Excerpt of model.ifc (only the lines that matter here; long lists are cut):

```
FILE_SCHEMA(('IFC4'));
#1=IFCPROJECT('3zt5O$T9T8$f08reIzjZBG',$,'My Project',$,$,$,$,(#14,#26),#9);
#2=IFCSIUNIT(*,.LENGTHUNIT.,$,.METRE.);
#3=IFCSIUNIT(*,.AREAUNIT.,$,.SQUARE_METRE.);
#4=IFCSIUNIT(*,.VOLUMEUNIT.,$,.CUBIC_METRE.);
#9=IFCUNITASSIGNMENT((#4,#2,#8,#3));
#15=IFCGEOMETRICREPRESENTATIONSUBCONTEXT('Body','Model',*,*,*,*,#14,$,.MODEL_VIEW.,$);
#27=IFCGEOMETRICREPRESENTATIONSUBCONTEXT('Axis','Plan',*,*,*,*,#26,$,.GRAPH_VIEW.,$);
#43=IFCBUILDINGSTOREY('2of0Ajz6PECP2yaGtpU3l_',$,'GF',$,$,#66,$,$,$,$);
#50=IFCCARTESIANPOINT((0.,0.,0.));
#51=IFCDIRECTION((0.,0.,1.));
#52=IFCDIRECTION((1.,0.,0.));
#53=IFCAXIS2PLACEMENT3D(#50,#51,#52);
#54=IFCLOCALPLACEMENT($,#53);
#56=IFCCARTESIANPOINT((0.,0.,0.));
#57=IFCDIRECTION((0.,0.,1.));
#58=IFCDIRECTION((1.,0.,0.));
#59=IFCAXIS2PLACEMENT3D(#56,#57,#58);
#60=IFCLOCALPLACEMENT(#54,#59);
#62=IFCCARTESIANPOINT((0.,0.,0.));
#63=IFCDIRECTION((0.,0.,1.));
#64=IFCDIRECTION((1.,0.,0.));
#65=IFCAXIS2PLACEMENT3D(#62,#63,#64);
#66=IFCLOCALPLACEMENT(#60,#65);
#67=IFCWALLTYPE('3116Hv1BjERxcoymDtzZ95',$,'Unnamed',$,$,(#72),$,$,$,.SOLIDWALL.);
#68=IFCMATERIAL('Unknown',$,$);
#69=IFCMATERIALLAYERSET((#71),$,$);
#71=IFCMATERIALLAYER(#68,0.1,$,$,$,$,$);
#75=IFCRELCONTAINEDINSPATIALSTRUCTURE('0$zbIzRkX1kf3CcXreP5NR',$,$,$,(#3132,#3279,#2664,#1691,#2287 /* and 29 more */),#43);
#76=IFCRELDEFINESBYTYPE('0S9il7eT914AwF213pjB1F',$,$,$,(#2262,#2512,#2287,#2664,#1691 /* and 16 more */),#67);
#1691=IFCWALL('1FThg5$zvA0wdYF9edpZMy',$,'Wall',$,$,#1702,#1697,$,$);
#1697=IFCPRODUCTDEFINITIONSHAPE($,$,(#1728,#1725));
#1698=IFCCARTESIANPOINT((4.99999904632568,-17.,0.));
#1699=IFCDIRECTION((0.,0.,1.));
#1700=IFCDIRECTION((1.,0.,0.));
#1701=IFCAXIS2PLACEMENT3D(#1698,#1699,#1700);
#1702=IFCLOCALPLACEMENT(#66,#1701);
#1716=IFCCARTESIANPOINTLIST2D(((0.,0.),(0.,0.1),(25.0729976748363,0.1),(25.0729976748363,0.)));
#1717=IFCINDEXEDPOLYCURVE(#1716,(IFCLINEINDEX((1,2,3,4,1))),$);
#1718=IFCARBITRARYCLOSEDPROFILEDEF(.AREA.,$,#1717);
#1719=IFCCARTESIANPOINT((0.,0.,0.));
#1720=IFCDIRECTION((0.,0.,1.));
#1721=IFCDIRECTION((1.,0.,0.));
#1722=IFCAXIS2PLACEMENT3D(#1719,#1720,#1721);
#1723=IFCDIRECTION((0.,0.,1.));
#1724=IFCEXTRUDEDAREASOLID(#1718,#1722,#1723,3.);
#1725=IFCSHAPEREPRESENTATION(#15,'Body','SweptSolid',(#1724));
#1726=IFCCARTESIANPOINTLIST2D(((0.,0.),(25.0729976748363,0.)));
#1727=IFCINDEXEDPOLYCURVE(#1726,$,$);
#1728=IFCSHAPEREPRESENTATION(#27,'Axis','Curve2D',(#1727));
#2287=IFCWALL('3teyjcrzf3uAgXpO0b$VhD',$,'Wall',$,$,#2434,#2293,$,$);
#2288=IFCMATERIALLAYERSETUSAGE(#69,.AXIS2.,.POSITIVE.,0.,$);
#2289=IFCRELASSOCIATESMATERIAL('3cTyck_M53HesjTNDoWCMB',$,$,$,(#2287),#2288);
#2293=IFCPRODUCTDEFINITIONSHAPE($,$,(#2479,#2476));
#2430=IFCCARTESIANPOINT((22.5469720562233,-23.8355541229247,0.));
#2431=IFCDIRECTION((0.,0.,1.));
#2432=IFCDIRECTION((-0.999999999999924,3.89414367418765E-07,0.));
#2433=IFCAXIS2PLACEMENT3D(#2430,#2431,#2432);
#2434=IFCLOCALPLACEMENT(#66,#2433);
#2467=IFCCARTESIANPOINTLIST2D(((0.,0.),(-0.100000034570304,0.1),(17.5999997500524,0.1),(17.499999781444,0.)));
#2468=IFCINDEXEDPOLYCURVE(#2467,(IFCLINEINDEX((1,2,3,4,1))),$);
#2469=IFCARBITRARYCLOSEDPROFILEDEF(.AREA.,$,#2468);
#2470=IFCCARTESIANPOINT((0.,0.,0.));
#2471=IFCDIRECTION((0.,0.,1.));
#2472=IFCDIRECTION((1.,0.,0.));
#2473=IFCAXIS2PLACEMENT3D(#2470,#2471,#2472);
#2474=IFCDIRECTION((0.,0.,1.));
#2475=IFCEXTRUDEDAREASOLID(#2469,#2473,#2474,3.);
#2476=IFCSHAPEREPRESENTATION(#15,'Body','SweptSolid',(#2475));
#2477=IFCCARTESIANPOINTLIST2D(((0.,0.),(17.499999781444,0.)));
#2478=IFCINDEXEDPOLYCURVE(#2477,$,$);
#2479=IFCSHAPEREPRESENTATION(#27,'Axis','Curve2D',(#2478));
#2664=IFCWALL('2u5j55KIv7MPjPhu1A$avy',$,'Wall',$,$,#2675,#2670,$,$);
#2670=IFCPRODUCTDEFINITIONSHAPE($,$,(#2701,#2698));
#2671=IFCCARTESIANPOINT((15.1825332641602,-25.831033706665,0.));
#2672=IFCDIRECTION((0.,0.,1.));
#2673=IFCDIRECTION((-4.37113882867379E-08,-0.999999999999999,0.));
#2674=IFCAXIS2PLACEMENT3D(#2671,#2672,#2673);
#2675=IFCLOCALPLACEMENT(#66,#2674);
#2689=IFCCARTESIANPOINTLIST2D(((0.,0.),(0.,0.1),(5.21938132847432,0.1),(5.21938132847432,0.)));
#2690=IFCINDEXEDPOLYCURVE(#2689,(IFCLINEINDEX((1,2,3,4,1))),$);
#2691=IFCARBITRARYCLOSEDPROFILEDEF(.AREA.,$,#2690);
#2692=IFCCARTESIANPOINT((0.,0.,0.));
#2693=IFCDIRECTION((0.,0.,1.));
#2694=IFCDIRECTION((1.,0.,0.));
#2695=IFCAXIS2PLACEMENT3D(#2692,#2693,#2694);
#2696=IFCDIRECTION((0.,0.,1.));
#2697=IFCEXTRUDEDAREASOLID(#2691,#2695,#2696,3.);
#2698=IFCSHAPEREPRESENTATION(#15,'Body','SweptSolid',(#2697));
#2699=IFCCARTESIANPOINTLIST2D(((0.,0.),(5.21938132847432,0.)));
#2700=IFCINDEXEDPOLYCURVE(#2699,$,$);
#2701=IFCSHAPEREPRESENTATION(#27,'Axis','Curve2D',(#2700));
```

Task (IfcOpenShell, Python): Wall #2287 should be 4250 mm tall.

```python
import ifcopenshell
import ifcopenshell.geom
import ifcopenshell.util.representation
import ifcopenshell.util.shape
import ifcopenshell.util.unit

model = ifcopenshell.open("model.ifc")
unit_scale = ifcopenshell.util.unit.calculate_unit_scale(model)
settings = ifcopenshell.geom.settings()


def volume(element):
    """Net volume in cubic metres, openings subtracted."""
    shape = ifcopenshell.geom.create_shape(settings, element)
    return ifcopenshell.util.shape.get_volume(shape.geometry)


wall = model.by_guid("3teyjcrzf3uAgXpO0b$VhD")
before = volume(wall)

body = ifcopenshell.util.representation.get_representation(wall, "Model", "Body")
solid = body.Items[0]
old_height = solid.Depth
solid.Depth = 4.25 / unit_scale
after = volume(wall)

print(f"height {old_height:g} -> {solid.Depth:g}, volume {before:.3f} -> {after:.3f} m3")

model.write("model_rev.ifc")
```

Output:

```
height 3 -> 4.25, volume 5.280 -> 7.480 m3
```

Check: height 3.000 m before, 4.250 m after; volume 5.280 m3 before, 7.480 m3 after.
